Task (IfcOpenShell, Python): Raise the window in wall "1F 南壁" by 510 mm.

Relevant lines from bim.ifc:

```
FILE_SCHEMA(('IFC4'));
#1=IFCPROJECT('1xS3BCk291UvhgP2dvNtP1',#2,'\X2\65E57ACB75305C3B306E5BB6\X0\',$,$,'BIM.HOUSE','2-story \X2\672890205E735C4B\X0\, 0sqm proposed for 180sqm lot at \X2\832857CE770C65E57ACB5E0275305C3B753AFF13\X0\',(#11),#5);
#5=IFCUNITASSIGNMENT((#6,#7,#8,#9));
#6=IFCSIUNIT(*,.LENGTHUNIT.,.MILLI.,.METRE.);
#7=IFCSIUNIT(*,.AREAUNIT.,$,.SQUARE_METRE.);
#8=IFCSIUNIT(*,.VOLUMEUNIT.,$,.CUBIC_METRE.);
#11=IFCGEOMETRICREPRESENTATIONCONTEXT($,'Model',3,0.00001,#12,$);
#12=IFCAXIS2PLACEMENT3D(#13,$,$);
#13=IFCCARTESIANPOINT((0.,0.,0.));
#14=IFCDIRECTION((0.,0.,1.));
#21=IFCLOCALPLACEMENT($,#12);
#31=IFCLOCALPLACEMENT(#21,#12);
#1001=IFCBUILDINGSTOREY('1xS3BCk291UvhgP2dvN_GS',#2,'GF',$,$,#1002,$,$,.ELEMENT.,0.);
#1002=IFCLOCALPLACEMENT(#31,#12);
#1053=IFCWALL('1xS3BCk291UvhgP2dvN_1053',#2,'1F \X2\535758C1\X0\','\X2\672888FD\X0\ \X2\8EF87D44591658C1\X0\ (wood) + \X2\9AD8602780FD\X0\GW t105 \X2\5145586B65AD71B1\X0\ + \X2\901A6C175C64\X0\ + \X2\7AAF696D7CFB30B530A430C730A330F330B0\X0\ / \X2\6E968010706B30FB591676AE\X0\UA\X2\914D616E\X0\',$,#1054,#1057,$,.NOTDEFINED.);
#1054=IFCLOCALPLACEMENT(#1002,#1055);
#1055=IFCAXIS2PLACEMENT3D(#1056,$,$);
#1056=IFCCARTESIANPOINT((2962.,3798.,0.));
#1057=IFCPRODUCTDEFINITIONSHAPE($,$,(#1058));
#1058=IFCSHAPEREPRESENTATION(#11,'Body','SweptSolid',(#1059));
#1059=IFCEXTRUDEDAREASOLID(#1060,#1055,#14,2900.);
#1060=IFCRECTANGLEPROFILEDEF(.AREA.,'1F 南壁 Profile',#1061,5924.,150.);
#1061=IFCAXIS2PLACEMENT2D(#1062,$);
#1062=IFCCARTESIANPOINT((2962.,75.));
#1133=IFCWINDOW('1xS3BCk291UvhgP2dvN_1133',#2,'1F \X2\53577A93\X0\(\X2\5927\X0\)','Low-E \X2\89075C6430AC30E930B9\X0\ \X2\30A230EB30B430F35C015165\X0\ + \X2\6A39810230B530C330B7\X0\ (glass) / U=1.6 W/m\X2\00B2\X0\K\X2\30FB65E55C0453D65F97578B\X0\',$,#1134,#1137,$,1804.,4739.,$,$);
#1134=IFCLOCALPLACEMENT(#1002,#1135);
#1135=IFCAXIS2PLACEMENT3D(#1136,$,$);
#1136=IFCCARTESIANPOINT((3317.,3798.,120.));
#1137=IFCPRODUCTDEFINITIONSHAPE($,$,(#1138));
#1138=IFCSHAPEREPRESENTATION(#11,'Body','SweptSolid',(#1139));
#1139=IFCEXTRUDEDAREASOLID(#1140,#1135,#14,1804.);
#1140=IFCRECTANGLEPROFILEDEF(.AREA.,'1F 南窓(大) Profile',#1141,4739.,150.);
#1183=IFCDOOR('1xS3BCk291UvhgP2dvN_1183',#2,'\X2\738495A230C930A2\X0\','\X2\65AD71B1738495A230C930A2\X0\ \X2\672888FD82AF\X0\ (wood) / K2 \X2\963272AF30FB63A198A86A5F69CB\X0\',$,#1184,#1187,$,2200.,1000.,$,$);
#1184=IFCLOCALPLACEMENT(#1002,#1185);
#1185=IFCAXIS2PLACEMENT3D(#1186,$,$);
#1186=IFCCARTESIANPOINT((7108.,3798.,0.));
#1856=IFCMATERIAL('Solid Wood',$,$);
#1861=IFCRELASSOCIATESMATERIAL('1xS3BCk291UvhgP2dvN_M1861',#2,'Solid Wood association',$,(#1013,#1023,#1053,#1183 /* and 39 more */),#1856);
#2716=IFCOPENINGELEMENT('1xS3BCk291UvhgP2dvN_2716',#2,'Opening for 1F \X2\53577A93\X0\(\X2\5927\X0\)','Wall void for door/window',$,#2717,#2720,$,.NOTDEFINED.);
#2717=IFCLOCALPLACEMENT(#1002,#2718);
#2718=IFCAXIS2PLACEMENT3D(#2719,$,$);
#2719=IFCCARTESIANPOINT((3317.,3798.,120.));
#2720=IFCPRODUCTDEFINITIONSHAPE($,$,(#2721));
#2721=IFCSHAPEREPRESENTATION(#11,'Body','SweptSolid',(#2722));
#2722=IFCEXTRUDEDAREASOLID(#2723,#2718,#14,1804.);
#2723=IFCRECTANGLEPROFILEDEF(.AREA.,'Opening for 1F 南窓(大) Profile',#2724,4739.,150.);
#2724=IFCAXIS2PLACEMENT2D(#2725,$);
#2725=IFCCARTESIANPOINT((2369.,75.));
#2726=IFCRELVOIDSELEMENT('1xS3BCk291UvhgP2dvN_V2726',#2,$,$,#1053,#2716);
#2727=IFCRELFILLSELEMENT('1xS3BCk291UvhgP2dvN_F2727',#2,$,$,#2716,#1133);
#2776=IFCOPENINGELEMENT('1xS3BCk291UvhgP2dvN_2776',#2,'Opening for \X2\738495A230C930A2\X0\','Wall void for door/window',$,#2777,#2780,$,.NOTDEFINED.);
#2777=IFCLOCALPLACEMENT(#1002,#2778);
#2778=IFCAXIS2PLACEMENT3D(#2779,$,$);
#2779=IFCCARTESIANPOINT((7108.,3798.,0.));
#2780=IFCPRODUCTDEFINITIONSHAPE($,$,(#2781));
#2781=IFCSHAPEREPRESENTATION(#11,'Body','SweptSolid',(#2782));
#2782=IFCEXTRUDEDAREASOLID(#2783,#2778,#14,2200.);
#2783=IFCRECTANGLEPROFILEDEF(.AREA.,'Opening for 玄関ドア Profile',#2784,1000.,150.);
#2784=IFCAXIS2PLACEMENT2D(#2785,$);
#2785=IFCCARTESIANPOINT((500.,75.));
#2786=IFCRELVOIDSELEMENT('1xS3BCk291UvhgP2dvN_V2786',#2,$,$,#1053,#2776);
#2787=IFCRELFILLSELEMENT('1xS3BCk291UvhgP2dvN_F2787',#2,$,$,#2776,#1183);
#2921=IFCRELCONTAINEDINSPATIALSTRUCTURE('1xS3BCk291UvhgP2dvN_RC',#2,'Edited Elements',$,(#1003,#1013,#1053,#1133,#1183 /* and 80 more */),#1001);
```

```python
import numpy as np
import ifcopenshell
import ifcopenshell.api.geometry
import ifcopenshell.util.placement
import ifcopenshell.util.unit

model = ifcopenshell.open("bim.ifc")
unit_scale = ifcopenshell.util.unit.calculate_unit_scale(model)

window = model.by_guid("1xS3BCk291UvhgP2dvN_1133")
opening = window.FillsVoids[0].RelatingOpeningElement
dz = 0.51 / unit_scale

shift = np.array([0.0, 0.0, dz])
# The window is not placed relative to its opening, so move both.
for product in (opening, window):
    matrix = ifcopenshell.util.placement.get_local_placement(product.ObjectPlacement)
    matrix[:3, 3] += shift
    ifcopenshell.api.geometry.edit_object_placement(model, product=product, matrix=matrix, is_si=False)

print(f"moved by {dz * unit_scale:+.3f} m")

model.write("bim_rev.ifc")
```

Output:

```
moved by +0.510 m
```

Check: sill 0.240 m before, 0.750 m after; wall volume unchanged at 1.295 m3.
